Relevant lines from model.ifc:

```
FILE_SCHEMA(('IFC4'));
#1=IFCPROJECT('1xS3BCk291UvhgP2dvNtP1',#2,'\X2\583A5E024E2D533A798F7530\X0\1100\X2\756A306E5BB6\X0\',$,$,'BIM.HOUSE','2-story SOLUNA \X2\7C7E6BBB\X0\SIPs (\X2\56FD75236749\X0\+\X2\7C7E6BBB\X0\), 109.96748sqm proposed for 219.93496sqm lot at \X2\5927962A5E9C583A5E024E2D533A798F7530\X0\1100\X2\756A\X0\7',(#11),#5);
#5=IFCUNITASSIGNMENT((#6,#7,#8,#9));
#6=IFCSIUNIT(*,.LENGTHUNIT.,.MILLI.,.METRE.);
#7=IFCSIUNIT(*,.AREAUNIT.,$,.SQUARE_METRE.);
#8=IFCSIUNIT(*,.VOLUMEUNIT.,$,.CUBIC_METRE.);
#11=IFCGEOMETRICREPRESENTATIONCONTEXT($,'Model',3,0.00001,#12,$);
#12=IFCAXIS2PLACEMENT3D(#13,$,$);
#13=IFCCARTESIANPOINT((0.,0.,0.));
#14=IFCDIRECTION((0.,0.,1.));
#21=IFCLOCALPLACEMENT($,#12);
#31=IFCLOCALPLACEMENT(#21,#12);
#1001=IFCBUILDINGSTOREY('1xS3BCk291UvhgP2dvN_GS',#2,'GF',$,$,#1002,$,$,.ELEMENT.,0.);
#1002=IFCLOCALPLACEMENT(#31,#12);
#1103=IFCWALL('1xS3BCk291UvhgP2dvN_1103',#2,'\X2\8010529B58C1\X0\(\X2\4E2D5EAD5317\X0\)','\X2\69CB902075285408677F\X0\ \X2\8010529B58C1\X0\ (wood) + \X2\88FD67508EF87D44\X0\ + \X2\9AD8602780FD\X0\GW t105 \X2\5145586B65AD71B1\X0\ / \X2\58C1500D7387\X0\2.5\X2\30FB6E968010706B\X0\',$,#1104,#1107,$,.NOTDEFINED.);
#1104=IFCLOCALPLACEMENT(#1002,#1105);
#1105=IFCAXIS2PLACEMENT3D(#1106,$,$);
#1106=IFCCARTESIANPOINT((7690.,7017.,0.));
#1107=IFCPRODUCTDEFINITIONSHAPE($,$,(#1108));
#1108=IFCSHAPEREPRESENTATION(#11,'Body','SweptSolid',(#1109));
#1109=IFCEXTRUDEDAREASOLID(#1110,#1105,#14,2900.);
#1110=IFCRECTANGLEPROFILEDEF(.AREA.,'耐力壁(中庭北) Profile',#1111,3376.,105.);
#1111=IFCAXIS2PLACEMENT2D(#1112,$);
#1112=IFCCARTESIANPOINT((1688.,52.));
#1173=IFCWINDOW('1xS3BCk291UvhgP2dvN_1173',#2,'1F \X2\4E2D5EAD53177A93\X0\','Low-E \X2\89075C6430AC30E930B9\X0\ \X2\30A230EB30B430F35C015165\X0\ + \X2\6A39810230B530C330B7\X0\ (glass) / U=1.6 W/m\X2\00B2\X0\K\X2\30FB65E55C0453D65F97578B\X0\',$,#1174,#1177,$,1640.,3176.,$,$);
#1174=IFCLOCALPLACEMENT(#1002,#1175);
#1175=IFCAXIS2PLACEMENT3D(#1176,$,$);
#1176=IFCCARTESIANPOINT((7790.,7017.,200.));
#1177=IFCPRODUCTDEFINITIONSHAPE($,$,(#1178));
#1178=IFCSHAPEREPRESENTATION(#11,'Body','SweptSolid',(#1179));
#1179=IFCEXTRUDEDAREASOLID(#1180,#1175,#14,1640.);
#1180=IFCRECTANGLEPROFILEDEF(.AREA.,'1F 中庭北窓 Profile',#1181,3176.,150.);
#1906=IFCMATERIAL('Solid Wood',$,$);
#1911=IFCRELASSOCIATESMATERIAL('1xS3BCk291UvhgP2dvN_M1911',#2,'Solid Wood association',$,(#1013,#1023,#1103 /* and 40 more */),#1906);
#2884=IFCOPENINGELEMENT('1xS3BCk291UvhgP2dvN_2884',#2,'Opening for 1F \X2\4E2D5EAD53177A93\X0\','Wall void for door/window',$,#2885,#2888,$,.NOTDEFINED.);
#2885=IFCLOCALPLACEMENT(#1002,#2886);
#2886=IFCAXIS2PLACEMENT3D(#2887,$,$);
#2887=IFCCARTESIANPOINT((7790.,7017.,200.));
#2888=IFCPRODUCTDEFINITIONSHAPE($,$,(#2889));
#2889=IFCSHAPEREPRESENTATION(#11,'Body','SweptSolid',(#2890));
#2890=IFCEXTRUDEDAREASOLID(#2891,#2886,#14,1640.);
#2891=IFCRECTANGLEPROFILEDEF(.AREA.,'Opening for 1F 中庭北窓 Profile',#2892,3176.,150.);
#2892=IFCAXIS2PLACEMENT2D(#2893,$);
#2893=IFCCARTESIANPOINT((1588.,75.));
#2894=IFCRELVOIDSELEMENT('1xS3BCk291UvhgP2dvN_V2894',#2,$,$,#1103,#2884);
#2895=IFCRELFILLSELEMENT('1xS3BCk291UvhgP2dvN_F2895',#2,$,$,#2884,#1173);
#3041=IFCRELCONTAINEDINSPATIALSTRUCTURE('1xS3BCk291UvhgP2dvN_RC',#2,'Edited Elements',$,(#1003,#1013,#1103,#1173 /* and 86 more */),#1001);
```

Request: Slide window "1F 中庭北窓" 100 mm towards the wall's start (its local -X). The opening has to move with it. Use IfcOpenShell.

```python
import ifcopenshell
import ifcopenshell.api.geometry
import ifcopenshell.util.placement

model = ifcopenshell.open("model.ifc")

window = model.by_id(1173)
opening = window.FillsVoids[0].RelatingOpeningElement
wall = opening.VoidsElements[0].RelatingBuildingElement

wall_matrix = ifcopenshell.util.placement.get_local_placement(wall.ObjectPlacement)
shift = wall_matrix[:3, 0] * -100.0
before = ifcopenshell.util.placement.get_local_placement(window.ObjectPlacement)[:3, 3].copy()

# The window is not placed relative to its opening, so move both.
for product in (opening, window):
    matrix = ifcopenshell.util.placement.get_local_placement(product.ObjectPlacement)
    matrix[:3, 3] += shift
    ifcopenshell.api.geometry.edit_object_placement(model, product=product, matrix=matrix, is_si=False)

after = ifcopenshell.util.placement.get_local_placement(window.ObjectPlacement)[:3, 3]
print("window moved by", (after - before).round(3) + 0.0)

model.write("model_updated.ifc")
```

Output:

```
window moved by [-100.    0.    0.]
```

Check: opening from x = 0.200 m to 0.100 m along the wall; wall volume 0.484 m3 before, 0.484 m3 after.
